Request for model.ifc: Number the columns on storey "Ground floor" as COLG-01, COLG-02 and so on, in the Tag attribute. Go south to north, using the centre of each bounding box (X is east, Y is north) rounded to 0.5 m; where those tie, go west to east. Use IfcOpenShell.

First a look at what the model holds.

```python
import ifcopenshell
import ifcopenshell.util.element
import ifcopenshell.util.placement

model = ifcopenshell.open("model.ifc")
print(model.schema)
storey = next(s for s in model.by_type("IfcBuildingStorey") if s.Name == "Ground floor")
columns = [e for e in ifcopenshell.util.element.get_decomposition(storey) if e.is_a("IfcColumn")]
for e in sorted(columns, key=lambda e: e.id()):
    origin = ifcopenshell.util.placement.get_local_placement(e.ObjectPlacement)[:3, 3]
    print(e.id(), e.Tag, e.Name, origin.round(2) + 0.0, sep=" | ")
```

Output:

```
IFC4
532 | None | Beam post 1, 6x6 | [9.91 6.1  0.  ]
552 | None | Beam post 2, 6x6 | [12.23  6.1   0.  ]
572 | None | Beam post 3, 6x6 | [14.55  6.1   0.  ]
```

```python
import ifcopenshell
import ifcopenshell.geom
import ifcopenshell.util.element
import ifcopenshell.util.shape

model = ifcopenshell.open("model.ifc")
settings = ifcopenshell.geom.settings()
settings.set("use-world-coords", True)


def centre(element):
    shape = ifcopenshell.geom.create_shape(settings, element)
    return ifcopenshell.util.shape.get_bbox_centroid(shape.geometry)


storey = next(s for s in model.by_type("IfcBuildingStorey") if s.Name == "Ground floor")
columns = [e for e in ifcopenshell.util.element.get_decomposition(storey) if e.is_a("IfcColumn")]

# Insertion points can sit at a corner or the storey origin, so sort by the geometry (in metres).
centres = {e: centre(e) for e in columns}
columns.sort(key=lambda e: (round(centres[e][1] / 0.5), centres[e][0]))

for i, e in enumerate(columns, start=1):
    number = f"COLG-{i:02d}"
    e.Tag = number
    print(e.id(), number)

model.write("model_updated.ifc")
```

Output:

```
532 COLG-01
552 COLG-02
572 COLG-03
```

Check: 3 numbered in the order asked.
